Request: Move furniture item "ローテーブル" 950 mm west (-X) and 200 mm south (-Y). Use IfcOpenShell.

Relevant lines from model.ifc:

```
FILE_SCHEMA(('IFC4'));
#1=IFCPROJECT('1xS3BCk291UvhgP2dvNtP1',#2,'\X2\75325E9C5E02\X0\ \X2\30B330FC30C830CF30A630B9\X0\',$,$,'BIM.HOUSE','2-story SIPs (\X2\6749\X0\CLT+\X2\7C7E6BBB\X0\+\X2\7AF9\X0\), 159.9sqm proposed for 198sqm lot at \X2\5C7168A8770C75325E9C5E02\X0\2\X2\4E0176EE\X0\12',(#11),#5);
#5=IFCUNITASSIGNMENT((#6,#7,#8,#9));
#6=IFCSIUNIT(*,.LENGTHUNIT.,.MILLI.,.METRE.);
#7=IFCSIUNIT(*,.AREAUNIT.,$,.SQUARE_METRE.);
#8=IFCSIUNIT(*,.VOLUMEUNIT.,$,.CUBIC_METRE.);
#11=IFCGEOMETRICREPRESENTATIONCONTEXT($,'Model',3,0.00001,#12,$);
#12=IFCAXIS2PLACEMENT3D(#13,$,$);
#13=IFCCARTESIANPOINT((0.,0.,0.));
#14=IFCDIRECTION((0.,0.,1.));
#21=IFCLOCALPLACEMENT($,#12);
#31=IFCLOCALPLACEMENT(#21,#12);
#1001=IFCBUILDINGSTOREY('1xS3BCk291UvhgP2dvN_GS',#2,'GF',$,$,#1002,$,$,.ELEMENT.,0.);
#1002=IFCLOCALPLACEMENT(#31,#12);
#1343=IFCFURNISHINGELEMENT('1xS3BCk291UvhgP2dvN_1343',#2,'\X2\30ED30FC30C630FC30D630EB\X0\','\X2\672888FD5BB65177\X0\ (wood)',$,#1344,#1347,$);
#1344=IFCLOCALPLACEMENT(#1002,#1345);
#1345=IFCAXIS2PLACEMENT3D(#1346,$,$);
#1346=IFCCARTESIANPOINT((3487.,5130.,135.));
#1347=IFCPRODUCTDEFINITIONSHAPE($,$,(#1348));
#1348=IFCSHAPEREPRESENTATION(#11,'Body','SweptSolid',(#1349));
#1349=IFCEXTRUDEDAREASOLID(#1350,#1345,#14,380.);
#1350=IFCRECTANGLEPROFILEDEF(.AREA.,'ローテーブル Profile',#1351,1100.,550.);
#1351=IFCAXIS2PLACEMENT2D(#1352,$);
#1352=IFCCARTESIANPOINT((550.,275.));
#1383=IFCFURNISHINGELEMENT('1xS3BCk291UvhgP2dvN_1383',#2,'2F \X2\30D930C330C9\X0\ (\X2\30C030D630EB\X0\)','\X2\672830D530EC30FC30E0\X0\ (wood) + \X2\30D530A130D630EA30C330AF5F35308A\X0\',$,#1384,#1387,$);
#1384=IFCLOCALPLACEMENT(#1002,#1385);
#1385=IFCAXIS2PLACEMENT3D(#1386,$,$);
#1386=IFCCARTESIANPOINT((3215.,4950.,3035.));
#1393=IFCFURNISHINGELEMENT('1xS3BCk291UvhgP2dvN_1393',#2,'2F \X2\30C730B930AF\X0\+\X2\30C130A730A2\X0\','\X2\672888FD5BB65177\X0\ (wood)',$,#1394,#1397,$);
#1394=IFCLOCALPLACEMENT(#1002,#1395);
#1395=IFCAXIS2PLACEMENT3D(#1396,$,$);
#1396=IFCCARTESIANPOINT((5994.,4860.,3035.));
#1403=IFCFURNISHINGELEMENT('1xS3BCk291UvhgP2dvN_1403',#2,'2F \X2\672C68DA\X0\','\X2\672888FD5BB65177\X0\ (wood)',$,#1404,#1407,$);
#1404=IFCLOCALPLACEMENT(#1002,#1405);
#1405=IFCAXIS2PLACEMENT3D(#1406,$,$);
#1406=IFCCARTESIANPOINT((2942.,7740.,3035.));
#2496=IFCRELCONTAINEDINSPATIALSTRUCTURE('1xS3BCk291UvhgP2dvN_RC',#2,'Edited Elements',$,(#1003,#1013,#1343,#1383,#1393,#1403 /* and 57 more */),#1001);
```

```python
import ifcopenshell
import ifcopenshell.api.geometry
import ifcopenshell.util.placement
import ifcopenshell.util.unit

model = ifcopenshell.open("model.ifc")
unit_scale = ifcopenshell.util.unit.calculate_unit_scale(model)

item = model.by_guid("1xS3BCk291UvhgP2dvN_1343")
matrix = ifcopenshell.util.placement.get_local_placement(item.ObjectPlacement)
matrix[0, 3] -= 0.95 / unit_scale
matrix[1, 3] -= 0.2 / unit_scale
ifcopenshell.api.geometry.edit_object_placement(model, product=item, matrix=matrix, is_si=False)

print(ifcopenshell.util.placement.get_local_placement(item.ObjectPlacement).round(3) + 0.0)

model.write("model_rev.ifc")
```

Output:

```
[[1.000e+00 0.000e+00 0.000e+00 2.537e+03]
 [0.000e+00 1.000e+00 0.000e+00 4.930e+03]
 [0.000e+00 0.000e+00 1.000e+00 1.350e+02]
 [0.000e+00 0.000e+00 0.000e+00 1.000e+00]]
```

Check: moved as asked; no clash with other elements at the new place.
